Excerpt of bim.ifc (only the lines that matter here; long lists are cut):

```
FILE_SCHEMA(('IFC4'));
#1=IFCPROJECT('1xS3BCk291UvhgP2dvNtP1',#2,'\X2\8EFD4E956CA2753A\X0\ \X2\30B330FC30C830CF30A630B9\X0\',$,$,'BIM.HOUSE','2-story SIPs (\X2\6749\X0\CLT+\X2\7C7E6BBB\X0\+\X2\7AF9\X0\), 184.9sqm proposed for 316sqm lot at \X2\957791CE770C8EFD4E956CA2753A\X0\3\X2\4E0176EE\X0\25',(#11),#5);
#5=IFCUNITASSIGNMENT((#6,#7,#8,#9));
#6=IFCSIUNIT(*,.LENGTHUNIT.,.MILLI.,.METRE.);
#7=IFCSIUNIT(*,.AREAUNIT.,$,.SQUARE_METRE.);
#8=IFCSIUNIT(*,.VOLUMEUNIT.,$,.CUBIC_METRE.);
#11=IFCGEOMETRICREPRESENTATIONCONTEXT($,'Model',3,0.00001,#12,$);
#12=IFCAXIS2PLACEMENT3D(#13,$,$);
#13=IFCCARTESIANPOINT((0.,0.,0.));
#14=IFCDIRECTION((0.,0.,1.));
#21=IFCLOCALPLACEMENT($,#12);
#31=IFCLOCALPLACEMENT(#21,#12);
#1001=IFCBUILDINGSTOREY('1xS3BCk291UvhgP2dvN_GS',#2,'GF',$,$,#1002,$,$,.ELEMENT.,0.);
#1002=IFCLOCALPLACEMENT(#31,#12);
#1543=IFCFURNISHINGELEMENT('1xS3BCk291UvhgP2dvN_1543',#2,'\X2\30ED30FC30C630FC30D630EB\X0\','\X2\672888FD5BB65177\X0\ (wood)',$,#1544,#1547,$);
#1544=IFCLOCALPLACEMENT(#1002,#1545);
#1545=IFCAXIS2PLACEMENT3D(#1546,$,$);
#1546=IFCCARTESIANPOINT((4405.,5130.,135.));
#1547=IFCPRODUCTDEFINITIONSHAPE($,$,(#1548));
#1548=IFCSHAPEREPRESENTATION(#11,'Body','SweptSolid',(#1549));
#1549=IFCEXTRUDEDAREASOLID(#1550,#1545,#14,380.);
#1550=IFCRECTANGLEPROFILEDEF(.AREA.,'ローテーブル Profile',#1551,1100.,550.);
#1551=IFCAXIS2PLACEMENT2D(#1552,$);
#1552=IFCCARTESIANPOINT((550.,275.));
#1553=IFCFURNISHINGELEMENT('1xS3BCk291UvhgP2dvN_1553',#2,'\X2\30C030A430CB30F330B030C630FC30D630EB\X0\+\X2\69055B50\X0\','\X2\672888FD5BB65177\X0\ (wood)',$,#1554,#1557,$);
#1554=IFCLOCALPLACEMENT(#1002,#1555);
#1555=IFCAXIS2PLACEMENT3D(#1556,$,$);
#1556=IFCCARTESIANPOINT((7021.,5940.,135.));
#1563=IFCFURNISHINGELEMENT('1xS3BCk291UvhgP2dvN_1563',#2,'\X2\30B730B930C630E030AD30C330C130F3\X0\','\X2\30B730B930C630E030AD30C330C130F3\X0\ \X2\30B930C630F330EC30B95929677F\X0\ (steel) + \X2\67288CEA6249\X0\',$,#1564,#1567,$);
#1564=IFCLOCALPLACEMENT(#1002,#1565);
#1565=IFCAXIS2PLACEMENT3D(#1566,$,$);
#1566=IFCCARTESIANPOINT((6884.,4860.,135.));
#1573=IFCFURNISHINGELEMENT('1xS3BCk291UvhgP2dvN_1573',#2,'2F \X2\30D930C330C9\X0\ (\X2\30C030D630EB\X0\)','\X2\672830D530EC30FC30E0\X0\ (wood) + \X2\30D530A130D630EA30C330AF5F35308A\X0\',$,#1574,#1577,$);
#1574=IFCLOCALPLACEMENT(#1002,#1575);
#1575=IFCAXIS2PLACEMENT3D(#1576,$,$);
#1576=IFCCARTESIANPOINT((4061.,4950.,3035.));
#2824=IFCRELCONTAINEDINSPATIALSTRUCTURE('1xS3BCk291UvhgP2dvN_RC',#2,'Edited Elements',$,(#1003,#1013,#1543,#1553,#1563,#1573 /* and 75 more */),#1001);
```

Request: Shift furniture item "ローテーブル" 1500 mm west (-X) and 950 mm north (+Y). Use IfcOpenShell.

```python
import ifcopenshell
import ifcopenshell.api.geometry
import ifcopenshell.util.placement

model = ifcopenshell.open("bim.ifc")

item = model.by_guid("1xS3BCk291UvhgP2dvN_1543")
matrix = ifcopenshell.util.placement.get_local_placement(item.ObjectPlacement)
matrix[0, 3] -= 1500.0
matrix[1, 3] += 950.0
ifcopenshell.api.geometry.edit_object_placement(model, product=item, matrix=matrix, is_si=False)

print(ifcopenshell.util.placement.get_local_placement(item.ObjectPlacement).round(3) + 0.0)

model.write("bim-out.ifc")
```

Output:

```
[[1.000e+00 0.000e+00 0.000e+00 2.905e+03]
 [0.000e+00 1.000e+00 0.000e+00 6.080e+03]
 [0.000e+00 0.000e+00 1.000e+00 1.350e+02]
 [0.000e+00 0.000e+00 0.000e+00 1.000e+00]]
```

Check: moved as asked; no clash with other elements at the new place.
